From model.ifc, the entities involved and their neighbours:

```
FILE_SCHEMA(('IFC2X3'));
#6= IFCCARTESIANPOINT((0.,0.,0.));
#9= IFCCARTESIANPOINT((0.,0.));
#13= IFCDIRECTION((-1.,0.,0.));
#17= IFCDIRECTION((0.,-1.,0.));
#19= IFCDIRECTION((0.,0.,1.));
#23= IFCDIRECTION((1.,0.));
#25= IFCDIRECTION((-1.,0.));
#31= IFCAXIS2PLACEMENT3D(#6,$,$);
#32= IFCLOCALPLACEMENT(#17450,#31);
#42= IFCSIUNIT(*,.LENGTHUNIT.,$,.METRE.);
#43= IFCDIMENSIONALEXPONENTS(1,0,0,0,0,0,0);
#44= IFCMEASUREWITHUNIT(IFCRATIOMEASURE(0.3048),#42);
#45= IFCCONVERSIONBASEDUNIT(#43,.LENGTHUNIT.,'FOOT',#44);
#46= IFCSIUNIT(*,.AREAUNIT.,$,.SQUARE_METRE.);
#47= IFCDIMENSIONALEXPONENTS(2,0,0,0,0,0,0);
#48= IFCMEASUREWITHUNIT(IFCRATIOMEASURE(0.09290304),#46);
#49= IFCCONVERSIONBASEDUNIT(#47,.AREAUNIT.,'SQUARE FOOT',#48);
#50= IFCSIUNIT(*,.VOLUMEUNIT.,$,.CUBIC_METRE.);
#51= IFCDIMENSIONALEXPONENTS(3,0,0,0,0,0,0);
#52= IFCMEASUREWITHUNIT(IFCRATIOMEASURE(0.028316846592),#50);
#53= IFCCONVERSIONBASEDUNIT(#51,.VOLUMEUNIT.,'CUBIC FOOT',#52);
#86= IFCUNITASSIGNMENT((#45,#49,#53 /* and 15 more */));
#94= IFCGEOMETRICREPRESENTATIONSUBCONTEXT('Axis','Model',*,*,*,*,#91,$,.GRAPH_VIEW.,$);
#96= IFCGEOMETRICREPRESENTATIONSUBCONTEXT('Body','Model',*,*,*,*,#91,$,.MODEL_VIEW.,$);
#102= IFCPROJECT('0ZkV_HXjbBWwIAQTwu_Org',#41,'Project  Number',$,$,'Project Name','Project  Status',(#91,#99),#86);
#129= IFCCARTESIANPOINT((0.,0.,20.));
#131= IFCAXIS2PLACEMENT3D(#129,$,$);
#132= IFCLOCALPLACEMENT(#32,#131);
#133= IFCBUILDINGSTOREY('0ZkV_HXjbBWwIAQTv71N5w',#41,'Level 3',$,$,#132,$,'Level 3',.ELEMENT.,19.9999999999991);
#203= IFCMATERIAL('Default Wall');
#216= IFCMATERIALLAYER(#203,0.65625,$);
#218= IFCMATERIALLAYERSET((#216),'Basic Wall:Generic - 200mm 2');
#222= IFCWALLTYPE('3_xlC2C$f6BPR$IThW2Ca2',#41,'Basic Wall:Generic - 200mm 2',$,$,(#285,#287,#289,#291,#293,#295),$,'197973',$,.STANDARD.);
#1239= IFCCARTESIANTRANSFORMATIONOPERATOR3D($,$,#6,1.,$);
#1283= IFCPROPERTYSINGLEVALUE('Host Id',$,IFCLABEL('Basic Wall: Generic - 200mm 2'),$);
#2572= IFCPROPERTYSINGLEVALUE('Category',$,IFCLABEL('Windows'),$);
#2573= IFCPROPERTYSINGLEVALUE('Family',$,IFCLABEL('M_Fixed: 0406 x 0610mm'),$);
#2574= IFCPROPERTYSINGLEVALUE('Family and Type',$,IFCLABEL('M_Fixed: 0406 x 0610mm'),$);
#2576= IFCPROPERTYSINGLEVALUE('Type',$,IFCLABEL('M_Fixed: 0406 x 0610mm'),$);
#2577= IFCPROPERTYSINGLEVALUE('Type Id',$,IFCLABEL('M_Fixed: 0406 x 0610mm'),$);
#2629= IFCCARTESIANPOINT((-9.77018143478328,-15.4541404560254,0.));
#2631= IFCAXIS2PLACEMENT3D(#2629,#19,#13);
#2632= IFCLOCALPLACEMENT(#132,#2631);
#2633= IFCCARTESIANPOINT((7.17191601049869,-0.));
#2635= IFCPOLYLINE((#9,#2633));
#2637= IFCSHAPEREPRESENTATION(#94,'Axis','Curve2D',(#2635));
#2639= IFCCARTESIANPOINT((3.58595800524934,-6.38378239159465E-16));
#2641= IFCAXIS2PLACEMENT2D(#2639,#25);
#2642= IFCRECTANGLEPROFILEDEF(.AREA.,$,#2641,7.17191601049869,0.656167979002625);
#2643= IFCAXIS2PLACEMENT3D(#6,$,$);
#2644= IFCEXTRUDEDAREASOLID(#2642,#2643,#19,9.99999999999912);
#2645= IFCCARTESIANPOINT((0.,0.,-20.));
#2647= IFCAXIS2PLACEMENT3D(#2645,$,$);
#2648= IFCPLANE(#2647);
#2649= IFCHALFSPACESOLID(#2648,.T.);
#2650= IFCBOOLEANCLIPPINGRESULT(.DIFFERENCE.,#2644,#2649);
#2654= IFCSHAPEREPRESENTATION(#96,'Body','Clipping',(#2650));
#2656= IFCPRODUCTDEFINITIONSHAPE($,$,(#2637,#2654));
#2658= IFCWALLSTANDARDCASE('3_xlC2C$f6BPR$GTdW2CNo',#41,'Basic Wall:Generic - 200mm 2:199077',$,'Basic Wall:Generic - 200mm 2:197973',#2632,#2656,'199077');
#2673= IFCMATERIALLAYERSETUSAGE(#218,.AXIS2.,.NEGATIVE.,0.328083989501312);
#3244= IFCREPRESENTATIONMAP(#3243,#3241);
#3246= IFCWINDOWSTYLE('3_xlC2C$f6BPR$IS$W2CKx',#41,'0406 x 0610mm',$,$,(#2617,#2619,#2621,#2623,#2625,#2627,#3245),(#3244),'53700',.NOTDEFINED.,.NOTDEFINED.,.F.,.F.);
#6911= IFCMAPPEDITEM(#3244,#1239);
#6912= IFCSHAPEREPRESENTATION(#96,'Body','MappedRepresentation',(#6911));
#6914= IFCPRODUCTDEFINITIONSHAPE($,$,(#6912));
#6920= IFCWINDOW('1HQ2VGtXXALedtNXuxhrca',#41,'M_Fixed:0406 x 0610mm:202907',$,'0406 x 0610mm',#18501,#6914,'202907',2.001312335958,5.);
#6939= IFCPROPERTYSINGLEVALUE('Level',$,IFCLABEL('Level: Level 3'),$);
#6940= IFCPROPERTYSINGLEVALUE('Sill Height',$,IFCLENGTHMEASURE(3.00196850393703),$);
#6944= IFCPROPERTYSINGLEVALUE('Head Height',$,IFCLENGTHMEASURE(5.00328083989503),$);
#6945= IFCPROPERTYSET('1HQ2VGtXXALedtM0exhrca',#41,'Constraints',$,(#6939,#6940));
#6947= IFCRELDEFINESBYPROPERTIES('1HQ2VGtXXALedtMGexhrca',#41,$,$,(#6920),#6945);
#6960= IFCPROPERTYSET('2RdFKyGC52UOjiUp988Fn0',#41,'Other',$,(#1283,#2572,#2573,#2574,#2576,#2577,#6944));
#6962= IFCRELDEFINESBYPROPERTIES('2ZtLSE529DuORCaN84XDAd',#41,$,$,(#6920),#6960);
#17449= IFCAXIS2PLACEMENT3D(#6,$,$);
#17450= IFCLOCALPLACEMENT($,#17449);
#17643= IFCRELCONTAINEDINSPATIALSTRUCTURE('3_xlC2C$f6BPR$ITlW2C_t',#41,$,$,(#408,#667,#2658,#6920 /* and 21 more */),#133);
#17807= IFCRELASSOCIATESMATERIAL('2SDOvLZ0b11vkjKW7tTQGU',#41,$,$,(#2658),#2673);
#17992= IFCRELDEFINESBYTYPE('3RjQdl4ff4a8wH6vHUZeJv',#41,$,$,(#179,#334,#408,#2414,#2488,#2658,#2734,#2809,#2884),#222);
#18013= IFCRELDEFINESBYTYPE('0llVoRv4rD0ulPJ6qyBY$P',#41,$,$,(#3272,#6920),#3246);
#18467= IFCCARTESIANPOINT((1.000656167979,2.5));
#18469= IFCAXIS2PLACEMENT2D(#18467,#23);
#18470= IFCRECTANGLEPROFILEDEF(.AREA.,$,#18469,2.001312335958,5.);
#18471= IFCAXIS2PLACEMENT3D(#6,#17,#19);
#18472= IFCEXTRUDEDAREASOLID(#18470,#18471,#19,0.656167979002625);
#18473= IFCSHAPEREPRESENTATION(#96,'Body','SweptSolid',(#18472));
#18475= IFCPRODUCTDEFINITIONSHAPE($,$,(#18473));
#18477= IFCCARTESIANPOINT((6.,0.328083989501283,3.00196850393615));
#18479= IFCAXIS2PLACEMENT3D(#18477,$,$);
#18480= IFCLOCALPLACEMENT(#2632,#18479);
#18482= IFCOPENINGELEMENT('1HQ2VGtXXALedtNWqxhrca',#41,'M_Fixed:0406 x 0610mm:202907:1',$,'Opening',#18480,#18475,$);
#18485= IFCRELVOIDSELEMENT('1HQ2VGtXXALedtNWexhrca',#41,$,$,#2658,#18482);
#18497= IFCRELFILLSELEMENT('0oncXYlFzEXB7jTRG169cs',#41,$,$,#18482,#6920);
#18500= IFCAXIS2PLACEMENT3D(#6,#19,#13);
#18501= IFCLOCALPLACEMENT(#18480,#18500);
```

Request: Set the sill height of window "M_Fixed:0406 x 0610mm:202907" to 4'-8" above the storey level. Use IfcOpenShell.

```python
import numpy as np
import ifcopenshell
import ifcopenshell.api.geometry
import ifcopenshell.api.pset
import ifcopenshell.geom
import ifcopenshell.util.element
import ifcopenshell.util.placement
import ifcopenshell.util.shape
import ifcopenshell.util.unit

model = ifcopenshell.open("model.ifc")
unit_scale = ifcopenshell.util.unit.calculate_unit_scale(model)

window = model.by_guid("1HQ2VGtXXALedtNXuxhrca")
opening = window.FillsVoids[0].RelatingOpeningElement
storey = ifcopenshell.util.element.get_container(window, ifc_class="IfcBuildingStorey")
level = ifcopenshell.util.placement.get_local_placement(storey.ObjectPlacement)[2, 3]

# The opening's origin need not be at the sill, so measure its lowest point.
shape = ifcopenshell.geom.create_shape(ifcopenshell.geom.settings(), opening)
bottom = ifcopenshell.util.shape.get_shape_bottom_elevation(shape, shape.geometry) / unit_scale
dz = level + 56 * 0.0254 / unit_scale - bottom

shift = np.array([0.0, 0.0, dz])
# The window is placed relative to its opening, so it follows when the opening moves.
matrix = ifcopenshell.util.placement.get_local_placement(opening.ObjectPlacement)
matrix[:3, 3] += shift
ifcopenshell.api.geometry.edit_object_placement(
    model, product=opening, matrix=matrix, is_si=False, should_transform_children=True
)

# Keep the stored heights in step.
pset = model.by_id(ifcopenshell.util.element.get_pset(window, "Constraints", should_inherit=False)["id"])
ifcopenshell.api.pset.edit_pset(model, pset=pset, properties={
    "Sill Height": model.create_entity("IfcLengthMeasure", ifcopenshell.util.element.get_pset(window, "Constraints", "Sill Height") + dz),
})
pset = model.by_id(ifcopenshell.util.element.get_pset(window, "Other", should_inherit=False)["id"])
ifcopenshell.api.pset.edit_pset(model, pset=pset, properties={
    "Head Height": model.create_entity("IfcLengthMeasure", ifcopenshell.util.element.get_pset(window, "Other", "Head Height") + dz),
})

print(f"moved by {dz * unit_scale:+.3f} m")

model.write("model_v2.ifc")
```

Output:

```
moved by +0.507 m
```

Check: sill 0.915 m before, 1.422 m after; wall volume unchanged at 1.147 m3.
